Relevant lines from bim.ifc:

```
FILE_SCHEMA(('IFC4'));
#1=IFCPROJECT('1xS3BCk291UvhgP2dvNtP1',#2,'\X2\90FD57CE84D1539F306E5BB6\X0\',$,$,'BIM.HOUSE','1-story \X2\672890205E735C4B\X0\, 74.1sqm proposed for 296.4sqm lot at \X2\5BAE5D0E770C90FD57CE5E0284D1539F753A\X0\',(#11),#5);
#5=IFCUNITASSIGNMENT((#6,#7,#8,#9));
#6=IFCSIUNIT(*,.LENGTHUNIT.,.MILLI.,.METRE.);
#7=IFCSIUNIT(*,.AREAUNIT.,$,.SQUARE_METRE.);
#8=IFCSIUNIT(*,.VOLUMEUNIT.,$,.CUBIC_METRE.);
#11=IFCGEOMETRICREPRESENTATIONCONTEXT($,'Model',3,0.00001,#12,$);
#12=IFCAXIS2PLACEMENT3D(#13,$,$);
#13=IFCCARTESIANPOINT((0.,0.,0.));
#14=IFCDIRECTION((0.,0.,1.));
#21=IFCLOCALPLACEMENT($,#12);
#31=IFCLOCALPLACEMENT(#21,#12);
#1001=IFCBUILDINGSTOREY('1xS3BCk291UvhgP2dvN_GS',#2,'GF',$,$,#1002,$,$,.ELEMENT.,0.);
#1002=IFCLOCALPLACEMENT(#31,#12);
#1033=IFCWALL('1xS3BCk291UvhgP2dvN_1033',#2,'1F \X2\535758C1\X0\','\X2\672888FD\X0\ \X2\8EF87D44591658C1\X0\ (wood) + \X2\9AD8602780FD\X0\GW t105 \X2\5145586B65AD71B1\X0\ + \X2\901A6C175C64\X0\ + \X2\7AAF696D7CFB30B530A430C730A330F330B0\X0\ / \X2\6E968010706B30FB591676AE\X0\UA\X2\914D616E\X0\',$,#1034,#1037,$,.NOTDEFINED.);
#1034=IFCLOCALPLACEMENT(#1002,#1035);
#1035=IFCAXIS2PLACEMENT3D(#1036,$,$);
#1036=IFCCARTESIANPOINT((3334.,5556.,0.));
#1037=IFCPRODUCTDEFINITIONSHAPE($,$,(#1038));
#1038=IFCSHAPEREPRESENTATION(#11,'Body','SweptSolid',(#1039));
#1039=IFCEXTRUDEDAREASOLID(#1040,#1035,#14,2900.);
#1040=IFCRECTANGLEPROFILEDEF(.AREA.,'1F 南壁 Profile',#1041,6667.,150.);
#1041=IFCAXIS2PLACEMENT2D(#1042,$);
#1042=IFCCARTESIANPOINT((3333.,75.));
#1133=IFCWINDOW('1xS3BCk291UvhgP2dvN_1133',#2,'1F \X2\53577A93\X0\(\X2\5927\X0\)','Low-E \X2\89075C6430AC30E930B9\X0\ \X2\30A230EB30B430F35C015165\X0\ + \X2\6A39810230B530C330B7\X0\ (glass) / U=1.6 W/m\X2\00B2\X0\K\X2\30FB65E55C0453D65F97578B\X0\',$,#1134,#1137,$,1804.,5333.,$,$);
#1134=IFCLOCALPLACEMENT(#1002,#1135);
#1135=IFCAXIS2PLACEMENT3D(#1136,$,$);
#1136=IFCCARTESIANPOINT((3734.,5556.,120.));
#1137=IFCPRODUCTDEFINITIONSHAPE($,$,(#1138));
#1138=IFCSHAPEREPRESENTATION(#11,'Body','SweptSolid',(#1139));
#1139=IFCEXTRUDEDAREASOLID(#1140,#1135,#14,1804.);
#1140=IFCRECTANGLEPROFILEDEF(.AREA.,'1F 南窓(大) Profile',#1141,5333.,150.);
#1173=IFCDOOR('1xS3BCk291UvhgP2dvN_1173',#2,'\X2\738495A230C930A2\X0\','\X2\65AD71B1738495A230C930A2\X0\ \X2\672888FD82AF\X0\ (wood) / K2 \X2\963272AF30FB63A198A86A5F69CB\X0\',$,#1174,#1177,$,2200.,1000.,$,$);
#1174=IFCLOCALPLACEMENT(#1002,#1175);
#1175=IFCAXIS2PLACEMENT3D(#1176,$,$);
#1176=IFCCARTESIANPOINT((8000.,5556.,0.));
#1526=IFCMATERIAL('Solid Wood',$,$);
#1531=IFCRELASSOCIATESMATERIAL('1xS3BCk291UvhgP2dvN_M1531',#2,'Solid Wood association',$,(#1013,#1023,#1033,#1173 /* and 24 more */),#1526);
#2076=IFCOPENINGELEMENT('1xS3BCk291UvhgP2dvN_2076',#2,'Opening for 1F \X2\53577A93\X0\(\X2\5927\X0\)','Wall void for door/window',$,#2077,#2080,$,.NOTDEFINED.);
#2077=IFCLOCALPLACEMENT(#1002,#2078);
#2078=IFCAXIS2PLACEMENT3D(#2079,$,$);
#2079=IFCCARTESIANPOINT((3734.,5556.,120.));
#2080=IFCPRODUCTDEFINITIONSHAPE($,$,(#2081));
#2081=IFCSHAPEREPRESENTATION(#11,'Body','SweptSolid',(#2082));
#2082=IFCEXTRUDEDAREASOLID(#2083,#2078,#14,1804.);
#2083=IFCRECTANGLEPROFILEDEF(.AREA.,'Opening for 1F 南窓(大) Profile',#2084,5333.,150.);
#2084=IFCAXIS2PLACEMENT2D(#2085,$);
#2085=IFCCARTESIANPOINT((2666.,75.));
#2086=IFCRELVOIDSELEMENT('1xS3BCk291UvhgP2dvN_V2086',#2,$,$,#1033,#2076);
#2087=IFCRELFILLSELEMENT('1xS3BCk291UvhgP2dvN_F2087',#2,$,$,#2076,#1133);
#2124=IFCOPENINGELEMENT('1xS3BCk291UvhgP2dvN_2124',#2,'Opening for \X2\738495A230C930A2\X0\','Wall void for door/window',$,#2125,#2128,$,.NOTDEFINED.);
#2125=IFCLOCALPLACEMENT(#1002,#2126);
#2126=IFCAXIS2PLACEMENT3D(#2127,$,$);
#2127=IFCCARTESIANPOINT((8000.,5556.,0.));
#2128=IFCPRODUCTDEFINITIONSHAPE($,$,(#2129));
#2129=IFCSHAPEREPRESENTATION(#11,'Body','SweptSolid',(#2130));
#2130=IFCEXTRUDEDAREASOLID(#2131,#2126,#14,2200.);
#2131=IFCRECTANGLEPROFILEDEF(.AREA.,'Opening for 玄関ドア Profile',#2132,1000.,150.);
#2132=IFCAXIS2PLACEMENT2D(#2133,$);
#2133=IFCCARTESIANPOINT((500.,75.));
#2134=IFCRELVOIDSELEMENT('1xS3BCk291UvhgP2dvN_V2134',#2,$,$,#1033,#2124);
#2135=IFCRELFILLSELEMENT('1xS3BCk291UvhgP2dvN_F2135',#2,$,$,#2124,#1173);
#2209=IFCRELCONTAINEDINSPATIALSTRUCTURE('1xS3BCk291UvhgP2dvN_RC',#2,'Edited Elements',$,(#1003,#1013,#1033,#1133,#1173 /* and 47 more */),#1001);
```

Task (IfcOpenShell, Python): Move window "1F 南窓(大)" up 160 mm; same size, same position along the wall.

```python
import numpy as np
import ifcopenshell
import ifcopenshell.api.geometry
import ifcopenshell.util.placement
import ifcopenshell.util.unit

model = ifcopenshell.open("bim.ifc")
unit_scale = ifcopenshell.util.unit.calculate_unit_scale(model)

window = model.by_guid("1xS3BCk291UvhgP2dvN_1133")
opening = window.FillsVoids[0].RelatingOpeningElement
dz = 160.0

shift = np.array([0.0, 0.0, dz])
# The window is not placed relative to its opening, so move both.
for product in (opening, window):
    matrix = ifcopenshell.util.placement.get_local_placement(product.ObjectPlacement)
    matrix[:3, 3] += shift
    ifcopenshell.api.geometry.edit_object_placement(model, product=product, matrix=matrix, is_si=False)

print(f"moved by {dz * unit_scale:+.3f} m")

model.write("bim_rev.ifc")
```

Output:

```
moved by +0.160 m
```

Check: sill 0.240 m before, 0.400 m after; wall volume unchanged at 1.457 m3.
